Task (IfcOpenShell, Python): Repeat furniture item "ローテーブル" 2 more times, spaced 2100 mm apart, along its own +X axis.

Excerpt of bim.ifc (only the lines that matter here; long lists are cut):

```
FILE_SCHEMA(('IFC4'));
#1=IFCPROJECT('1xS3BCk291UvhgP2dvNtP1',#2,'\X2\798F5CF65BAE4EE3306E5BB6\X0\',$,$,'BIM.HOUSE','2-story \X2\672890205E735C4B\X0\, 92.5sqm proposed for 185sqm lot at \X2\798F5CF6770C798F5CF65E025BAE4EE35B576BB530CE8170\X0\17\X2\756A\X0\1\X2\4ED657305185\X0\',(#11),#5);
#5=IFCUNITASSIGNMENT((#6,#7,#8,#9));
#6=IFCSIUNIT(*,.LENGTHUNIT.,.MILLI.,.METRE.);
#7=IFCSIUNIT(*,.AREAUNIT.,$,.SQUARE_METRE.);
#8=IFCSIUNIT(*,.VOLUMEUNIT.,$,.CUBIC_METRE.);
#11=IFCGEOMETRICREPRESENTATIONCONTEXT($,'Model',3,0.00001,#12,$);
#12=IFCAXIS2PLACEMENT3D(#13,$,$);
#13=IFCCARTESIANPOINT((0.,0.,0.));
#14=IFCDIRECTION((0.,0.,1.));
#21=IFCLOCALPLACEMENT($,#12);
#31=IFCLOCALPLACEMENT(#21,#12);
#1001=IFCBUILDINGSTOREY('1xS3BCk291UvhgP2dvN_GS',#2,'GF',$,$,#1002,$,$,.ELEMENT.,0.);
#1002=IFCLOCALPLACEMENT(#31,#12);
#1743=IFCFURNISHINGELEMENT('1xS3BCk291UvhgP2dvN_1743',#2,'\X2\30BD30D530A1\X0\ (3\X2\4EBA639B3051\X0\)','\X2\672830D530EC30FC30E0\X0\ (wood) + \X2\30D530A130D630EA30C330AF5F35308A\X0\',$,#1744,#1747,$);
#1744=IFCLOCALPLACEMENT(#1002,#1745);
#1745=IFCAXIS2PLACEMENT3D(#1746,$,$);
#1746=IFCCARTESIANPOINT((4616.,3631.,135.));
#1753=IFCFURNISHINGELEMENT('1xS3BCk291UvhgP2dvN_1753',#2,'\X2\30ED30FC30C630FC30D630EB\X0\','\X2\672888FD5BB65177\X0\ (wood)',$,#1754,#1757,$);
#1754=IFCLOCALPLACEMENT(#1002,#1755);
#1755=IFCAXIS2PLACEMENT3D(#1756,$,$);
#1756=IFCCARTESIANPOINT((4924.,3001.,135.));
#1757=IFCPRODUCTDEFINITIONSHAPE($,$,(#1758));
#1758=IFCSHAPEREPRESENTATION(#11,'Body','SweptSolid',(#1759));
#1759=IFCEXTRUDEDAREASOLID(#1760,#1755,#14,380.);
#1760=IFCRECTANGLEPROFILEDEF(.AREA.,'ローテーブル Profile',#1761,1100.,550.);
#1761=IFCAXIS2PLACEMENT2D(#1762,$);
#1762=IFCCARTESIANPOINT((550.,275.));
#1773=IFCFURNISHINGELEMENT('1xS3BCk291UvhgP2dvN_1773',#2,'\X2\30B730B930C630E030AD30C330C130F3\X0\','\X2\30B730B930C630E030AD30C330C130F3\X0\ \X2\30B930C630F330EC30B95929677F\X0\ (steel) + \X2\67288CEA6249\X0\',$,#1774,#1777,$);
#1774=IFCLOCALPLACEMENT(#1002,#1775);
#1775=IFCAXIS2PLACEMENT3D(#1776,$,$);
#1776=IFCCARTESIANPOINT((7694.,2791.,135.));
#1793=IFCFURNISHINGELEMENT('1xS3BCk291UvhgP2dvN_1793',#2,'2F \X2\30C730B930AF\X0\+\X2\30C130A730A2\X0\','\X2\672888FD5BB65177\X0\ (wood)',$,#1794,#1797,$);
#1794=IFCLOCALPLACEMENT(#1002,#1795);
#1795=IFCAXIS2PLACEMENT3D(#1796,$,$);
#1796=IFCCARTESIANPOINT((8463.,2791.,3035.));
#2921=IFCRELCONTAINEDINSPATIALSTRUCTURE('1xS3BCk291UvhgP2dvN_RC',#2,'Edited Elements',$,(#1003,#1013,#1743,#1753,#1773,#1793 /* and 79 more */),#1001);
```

```python
import ifcopenshell
import ifcopenshell.api.geometry
import ifcopenshell.api.root
import ifcopenshell.util.element
import ifcopenshell.util.placement
import ifcopenshell.util.unit

model = ifcopenshell.open("bim.ifc")
unit_scale = ifcopenshell.util.unit.calculate_unit_scale(model)


def reuse_history(source, copy):
    """copy_class also copies each property set's owner history, people and application; keep the originals."""
    for rel in copy.IsDefinedBy:
        if rel.is_a("IfcRelDefinesByProperties") and (history := rel.RelatingPropertyDefinition.OwnerHistory):
            rel.RelatingPropertyDefinition.OwnerHistory = source.OwnerHistory
            ifcopenshell.util.element.remove_deep2(model, history)


source = model.by_guid("1xS3BCk291UvhgP2dvN_1753")
base = ifcopenshell.util.placement.get_local_placement(source.ObjectPlacement)
step = base[:3, 0] * 2.1 / unit_scale

for i in range(1, 3):
    copy = ifcopenshell.api.root.copy_class(model, product=source)
    copy.Representation = ifcopenshell.util.element.copy_deep(
        model, source.Representation, exclude=["IfcGeometricRepresentationContext", "IfcRepresentationMap"]
    )
    reuse_history(source, copy)
    matrix = base.copy()
    matrix[:3, 3] += i * step
    print("added at", matrix[:3, 3].round(3) + 0.0)
    ifcopenshell.api.geometry.edit_object_placement(model, product=copy, matrix=matrix, is_si=False)

model.write("bim_edited.ifc")
```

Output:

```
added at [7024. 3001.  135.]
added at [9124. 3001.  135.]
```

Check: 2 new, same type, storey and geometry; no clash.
